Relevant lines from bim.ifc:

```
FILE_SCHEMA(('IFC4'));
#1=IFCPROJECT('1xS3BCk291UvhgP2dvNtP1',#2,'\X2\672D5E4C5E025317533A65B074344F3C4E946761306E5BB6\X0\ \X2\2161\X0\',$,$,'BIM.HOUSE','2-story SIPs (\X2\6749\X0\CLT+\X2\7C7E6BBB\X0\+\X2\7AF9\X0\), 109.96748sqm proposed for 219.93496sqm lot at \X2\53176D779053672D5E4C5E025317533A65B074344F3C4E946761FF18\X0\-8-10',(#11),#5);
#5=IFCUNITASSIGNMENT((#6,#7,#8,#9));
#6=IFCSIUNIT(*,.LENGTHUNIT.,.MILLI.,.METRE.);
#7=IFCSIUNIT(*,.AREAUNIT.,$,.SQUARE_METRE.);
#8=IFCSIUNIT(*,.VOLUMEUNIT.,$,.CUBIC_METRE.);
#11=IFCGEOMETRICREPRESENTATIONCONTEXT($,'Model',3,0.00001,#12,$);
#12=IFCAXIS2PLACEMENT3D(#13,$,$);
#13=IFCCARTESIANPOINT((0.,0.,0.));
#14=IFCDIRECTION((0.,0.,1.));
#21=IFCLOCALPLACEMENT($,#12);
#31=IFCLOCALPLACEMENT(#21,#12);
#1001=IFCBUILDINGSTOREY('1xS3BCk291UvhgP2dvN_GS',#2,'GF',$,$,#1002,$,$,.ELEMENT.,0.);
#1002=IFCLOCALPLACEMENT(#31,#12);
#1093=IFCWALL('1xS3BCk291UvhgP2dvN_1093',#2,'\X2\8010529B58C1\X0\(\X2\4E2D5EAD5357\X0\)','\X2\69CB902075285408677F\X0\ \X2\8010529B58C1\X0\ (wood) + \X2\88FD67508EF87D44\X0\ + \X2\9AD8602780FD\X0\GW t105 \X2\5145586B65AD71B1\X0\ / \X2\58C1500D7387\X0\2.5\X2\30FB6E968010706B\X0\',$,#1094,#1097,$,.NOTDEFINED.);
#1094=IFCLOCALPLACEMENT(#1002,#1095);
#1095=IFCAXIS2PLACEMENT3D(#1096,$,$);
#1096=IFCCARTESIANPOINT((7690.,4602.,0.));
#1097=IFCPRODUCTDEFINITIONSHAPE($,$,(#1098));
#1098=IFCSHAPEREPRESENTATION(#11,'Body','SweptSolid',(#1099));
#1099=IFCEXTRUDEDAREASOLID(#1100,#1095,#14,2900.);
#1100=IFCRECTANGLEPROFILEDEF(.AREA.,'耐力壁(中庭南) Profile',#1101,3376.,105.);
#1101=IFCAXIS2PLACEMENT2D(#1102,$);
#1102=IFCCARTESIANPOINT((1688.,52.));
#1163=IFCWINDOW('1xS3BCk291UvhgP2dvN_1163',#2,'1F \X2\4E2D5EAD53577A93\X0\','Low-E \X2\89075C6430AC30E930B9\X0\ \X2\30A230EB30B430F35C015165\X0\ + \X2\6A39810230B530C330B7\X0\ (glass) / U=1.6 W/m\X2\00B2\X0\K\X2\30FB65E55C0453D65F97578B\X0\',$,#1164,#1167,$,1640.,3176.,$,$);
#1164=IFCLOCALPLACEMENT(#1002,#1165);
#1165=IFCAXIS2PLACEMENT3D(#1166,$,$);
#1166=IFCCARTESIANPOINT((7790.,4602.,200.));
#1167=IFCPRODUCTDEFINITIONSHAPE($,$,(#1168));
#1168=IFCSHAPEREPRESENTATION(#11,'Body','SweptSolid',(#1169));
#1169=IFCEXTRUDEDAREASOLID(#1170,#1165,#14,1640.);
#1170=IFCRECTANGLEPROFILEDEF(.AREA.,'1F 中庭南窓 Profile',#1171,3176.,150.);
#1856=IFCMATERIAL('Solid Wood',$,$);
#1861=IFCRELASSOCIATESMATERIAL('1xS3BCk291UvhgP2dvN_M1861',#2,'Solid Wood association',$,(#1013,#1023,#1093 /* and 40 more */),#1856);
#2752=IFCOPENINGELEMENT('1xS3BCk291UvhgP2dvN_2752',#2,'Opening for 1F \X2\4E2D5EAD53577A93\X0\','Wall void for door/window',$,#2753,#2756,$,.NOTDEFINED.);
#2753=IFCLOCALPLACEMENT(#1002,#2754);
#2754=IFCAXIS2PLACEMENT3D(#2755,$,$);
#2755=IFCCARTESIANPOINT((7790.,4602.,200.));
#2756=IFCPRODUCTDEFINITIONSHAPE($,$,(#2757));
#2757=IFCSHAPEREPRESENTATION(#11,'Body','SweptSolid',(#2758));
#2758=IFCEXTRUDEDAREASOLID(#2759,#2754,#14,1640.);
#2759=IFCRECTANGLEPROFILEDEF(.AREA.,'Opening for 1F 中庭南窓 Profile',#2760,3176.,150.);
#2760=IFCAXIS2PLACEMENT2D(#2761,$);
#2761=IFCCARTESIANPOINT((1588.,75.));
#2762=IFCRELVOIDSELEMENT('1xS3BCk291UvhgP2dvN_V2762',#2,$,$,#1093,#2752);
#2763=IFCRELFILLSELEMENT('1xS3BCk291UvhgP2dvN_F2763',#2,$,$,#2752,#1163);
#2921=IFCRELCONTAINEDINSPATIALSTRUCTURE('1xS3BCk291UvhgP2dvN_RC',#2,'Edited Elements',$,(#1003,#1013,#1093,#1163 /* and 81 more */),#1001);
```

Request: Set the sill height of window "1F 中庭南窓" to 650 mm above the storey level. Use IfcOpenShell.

```python
import numpy as np
import ifcopenshell
import ifcopenshell.api.geometry
import ifcopenshell.geom
import ifcopenshell.util.element
import ifcopenshell.util.placement
import ifcopenshell.util.shape
import ifcopenshell.util.unit

model = ifcopenshell.open("bim.ifc")
unit_scale = ifcopenshell.util.unit.calculate_unit_scale(model)

window = model.by_id(1163)
opening = window.FillsVoids[0].RelatingOpeningElement
storey = ifcopenshell.util.element.get_container(window, ifc_class="IfcBuildingStorey")
level = ifcopenshell.util.placement.get_local_placement(storey.ObjectPlacement)[2, 3]

# The opening's origin need not be at the sill, so measure its lowest point.
shape = ifcopenshell.geom.create_shape(ifcopenshell.geom.settings(), opening)
bottom = ifcopenshell.util.shape.get_shape_bottom_elevation(shape, shape.geometry) / unit_scale
dz = level + 650.0 - bottom

shift = np.array([0.0, 0.0, dz])
# The window is not placed relative to its opening, so move both.
for product in (opening, window):
    matrix = ifcopenshell.util.placement.get_local_placement(product.ObjectPlacement)
    matrix[:3, 3] += shift
    ifcopenshell.api.geometry.edit_object_placement(model, product=product, matrix=matrix, is_si=False)

print(f"moved by {dz * unit_scale:+.3f} m")

model.write("bim_edited.ifc")
```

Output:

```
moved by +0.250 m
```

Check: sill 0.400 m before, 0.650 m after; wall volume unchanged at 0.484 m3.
